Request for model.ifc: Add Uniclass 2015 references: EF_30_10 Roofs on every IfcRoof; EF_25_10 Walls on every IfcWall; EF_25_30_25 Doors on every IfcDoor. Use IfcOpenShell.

First a look at what the model holds.

```python
import ifcopenshell

model = ifcopenshell.open("model.ifc")
print(model.schema)
print("classifications:", [c.Name for c in model.by_type("IfcClassification")])
for ifc_class in ("IfcDoor", "IfcRoof", "IfcStair", "IfcWall", "IfcWindow"):
    print(ifc_class, len(model.by_type(ifc_class)))
```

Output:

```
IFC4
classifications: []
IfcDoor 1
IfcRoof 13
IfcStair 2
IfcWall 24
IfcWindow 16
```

```python
import ifcopenshell
import ifcopenshell.api.classification

model = ifcopenshell.open("model.ifc")

system = ifcopenshell.api.classification.add_classification(model, classification="Uniclass 2015")

codes = {
    "IfcRoof": ("EF_30_10", "Roofs"),
    "IfcWall": ("EF_25_10", "Walls"),
    "IfcDoor": ("EF_25_30_25", "Doors"),
}
for ifc_class, (code, name) in codes.items():
    products = model.by_type(ifc_class)
    ifcopenshell.api.classification.add_reference(
        model, products=products, classification=system, identification=code, name=name
    )
    print(code, len(products))

model.write("model_updated.ifc")
```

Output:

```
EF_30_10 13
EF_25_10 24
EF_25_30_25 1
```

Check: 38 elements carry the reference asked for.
